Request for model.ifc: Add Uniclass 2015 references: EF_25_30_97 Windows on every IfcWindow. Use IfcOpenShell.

First a look at what the model holds.

```python
import ifcopenshell

model = ifcopenshell.open("model.ifc")
print(model.schema)
print("classifications:", [c.Name for c in model.by_type("IfcClassification")])
for ifc_class in ("IfcDoor", "IfcRoof", "IfcStair", "IfcWall", "IfcWindow"):
    print(ifc_class, len(model.by_type(ifc_class)))
```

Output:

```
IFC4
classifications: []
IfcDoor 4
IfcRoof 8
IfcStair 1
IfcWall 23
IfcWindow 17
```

```python
import ifcopenshell
import ifcopenshell.api.classification

model = ifcopenshell.open("model.ifc")

system = ifcopenshell.api.classification.add_classification(model, classification="Uniclass 2015")

codes = {
    "IfcWindow": ("EF_25_30_97", "Windows"),
}
for ifc_class, (code, name) in codes.items():
    products = model.by_type(ifc_class)
    ifcopenshell.api.classification.add_reference(
        model, products=products, classification=system, identification=code, name=name
    )
    print(code, len(products))

model.write("model_updated.ifc")
```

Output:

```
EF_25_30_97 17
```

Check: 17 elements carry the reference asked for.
